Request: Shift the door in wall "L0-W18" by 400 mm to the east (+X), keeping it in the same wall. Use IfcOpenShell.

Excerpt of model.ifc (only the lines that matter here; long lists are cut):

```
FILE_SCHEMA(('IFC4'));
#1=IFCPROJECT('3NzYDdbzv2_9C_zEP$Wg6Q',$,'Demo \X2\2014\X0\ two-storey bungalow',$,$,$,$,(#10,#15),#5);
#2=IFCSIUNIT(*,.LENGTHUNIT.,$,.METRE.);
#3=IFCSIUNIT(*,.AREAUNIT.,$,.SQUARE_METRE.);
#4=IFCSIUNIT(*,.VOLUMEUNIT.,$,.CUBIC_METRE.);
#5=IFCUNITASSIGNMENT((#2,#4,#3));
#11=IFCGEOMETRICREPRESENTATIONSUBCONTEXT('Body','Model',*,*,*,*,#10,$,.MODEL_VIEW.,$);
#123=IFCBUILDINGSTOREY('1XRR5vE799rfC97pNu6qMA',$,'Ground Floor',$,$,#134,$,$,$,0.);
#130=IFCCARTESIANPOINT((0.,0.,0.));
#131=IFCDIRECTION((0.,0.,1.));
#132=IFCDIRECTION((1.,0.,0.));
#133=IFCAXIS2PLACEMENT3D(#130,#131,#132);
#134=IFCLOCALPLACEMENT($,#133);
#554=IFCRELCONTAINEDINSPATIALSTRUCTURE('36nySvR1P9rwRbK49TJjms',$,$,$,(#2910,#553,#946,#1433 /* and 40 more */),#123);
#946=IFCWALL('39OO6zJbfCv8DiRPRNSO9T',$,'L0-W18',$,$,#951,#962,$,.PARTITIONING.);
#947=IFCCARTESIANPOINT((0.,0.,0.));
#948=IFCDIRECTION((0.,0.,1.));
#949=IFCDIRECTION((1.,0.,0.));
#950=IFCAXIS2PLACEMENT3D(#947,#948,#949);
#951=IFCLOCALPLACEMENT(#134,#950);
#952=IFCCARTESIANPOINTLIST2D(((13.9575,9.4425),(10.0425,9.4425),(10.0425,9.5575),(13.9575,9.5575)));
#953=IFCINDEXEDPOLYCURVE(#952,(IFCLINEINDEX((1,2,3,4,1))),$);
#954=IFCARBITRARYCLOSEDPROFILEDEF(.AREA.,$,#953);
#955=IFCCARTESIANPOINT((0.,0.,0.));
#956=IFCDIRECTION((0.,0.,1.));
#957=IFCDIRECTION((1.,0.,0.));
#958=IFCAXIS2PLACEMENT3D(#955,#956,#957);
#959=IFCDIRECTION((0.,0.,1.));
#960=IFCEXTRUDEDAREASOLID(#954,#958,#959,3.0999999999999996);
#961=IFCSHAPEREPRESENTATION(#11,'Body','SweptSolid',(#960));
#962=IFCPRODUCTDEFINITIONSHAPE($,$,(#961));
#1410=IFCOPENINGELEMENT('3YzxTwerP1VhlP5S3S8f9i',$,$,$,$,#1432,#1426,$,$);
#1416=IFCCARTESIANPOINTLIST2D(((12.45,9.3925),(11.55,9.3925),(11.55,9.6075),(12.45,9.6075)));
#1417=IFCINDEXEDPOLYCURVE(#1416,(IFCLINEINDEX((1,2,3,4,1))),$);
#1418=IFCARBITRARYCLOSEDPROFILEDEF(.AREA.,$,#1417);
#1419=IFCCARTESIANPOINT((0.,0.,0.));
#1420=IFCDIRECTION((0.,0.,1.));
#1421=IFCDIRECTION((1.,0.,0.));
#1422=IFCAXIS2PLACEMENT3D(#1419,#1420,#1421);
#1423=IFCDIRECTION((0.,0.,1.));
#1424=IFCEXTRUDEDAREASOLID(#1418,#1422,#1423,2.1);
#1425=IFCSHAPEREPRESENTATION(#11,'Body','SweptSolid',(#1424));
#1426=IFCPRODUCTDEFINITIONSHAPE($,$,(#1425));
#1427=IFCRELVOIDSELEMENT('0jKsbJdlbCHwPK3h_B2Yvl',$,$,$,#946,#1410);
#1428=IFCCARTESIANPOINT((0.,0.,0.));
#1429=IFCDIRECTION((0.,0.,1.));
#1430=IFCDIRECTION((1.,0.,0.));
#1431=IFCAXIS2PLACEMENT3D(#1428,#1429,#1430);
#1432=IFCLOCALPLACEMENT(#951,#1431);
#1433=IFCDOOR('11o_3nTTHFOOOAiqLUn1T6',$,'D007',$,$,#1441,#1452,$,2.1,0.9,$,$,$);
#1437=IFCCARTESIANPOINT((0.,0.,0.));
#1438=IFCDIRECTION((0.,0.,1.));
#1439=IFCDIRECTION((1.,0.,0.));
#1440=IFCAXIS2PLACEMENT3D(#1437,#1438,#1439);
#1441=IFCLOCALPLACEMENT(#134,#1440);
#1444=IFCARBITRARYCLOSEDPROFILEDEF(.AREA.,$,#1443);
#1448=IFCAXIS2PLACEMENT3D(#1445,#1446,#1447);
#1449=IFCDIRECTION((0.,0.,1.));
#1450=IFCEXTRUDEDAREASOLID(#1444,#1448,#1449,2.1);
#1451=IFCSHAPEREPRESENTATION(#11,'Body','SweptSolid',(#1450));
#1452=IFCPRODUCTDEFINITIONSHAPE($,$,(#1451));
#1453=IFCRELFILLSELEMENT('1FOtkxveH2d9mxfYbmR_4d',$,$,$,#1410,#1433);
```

```python
import ifcopenshell
import ifcopenshell.api.geometry
import ifcopenshell.util.placement

model = ifcopenshell.open("model.ifc")

door = model.by_guid("11o_3nTTHFOOOAiqLUn1T6")
opening = door.FillsVoids[0].RelatingOpeningElement
wall = opening.VoidsElements[0].RelatingBuildingElement

wall_matrix = ifcopenshell.util.placement.get_local_placement(wall.ObjectPlacement)
shift = wall_matrix[:3, 0] * 0.4
before = ifcopenshell.util.placement.get_local_placement(door.ObjectPlacement)[:3, 3].copy()

# The door is not placed relative to its opening, so move both.
for product in (opening, door):
    matrix = ifcopenshell.util.placement.get_local_placement(product.ObjectPlacement)
    matrix[:3, 3] += shift
    ifcopenshell.api.geometry.edit_object_placement(model, product=product, matrix=matrix, is_si=False)

after = ifcopenshell.util.placement.get_local_placement(door.ObjectPlacement)[:3, 3]
print("door moved by", (after - before).round(3) + 0.0)

model.write("model_rev.ifc")
```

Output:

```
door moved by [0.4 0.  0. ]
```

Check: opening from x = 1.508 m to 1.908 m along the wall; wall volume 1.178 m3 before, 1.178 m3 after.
